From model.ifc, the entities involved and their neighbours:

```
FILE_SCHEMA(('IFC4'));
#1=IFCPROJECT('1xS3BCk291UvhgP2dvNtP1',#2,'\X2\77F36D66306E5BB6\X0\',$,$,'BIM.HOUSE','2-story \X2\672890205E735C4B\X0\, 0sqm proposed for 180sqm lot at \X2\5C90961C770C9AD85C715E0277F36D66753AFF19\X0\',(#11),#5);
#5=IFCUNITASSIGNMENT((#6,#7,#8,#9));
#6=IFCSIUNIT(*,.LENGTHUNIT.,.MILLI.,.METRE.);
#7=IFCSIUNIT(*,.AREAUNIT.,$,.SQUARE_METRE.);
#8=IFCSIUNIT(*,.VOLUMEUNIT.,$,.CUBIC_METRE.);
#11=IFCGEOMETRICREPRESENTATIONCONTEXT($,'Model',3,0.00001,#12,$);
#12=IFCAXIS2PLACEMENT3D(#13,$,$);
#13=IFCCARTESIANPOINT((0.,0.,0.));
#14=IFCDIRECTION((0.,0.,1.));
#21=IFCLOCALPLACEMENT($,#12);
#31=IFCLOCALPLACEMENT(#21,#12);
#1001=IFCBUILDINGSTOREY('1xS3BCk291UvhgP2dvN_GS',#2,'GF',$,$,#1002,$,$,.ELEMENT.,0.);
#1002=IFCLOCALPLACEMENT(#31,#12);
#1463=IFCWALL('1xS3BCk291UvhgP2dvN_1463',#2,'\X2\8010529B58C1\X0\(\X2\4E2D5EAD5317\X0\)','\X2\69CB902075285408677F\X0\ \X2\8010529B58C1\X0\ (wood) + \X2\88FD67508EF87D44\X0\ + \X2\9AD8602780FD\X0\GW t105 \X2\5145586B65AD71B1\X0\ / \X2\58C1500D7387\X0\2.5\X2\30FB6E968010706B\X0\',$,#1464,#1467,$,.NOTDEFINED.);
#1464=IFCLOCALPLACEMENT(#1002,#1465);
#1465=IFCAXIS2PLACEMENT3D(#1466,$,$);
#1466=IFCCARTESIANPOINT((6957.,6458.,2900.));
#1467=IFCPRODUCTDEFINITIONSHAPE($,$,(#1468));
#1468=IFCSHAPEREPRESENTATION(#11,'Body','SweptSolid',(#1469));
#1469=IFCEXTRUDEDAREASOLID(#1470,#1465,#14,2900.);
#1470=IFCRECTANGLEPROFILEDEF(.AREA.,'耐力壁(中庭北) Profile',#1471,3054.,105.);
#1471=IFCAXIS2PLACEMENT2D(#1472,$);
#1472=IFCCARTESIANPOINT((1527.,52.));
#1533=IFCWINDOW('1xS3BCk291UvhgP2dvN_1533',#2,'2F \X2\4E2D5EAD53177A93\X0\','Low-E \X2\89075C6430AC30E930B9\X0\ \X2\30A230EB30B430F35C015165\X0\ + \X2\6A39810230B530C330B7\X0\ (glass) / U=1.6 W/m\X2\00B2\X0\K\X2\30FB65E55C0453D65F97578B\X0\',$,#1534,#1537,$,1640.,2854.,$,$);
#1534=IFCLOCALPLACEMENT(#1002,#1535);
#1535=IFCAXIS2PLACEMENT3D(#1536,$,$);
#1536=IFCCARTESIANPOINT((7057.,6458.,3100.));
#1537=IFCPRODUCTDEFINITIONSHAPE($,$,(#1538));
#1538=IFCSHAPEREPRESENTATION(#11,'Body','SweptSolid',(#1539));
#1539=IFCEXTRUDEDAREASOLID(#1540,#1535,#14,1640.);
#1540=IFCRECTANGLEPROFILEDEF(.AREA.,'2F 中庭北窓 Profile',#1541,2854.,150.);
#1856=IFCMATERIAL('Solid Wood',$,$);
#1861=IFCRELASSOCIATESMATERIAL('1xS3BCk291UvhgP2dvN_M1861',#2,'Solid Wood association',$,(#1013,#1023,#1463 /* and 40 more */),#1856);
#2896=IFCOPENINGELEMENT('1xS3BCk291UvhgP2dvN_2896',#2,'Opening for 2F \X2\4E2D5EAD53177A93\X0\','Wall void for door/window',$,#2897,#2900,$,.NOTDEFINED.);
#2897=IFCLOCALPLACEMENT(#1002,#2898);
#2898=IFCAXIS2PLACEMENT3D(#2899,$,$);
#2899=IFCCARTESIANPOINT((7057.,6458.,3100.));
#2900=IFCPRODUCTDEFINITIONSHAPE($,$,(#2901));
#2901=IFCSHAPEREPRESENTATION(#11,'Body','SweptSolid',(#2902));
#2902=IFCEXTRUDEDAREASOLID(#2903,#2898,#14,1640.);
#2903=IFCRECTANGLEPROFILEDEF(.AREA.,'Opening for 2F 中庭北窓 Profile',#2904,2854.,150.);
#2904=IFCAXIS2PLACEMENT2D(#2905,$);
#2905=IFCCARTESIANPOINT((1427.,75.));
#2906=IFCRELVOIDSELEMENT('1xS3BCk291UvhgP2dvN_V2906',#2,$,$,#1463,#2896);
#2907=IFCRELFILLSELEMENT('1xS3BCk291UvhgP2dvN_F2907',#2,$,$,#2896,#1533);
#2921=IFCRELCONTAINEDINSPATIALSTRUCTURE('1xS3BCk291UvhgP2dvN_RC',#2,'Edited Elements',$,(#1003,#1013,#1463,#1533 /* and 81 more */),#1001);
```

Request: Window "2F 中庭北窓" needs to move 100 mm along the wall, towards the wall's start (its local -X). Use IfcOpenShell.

```python
import ifcopenshell
import ifcopenshell.api.geometry
import ifcopenshell.util.placement
import ifcopenshell.util.unit

model = ifcopenshell.open("model.ifc")
unit_scale = ifcopenshell.util.unit.calculate_unit_scale(model)

window = model.by_id(1533)
opening = window.FillsVoids[0].RelatingOpeningElement
wall = opening.VoidsElements[0].RelatingBuildingElement

wall_matrix = ifcopenshell.util.placement.get_local_placement(wall.ObjectPlacement)
shift = wall_matrix[:3, 0] * -0.1 / unit_scale
before = ifcopenshell.util.placement.get_local_placement(window.ObjectPlacement)[:3, 3].copy()

# The window is not placed relative to its opening, so move both.
for product in (opening, window):
    matrix = ifcopenshell.util.placement.get_local_placement(product.ObjectPlacement)
    matrix[:3, 3] += shift
    ifcopenshell.api.geometry.edit_object_placement(model, product=product, matrix=matrix, is_si=False)

after = ifcopenshell.util.placement.get_local_placement(window.ObjectPlacement)[:3, 3]
print("window moved by", (after - before).round(3) + 0.0)

model.write("model_edited.ifc")
```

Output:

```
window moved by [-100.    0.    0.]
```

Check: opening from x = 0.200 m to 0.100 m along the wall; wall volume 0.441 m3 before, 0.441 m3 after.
